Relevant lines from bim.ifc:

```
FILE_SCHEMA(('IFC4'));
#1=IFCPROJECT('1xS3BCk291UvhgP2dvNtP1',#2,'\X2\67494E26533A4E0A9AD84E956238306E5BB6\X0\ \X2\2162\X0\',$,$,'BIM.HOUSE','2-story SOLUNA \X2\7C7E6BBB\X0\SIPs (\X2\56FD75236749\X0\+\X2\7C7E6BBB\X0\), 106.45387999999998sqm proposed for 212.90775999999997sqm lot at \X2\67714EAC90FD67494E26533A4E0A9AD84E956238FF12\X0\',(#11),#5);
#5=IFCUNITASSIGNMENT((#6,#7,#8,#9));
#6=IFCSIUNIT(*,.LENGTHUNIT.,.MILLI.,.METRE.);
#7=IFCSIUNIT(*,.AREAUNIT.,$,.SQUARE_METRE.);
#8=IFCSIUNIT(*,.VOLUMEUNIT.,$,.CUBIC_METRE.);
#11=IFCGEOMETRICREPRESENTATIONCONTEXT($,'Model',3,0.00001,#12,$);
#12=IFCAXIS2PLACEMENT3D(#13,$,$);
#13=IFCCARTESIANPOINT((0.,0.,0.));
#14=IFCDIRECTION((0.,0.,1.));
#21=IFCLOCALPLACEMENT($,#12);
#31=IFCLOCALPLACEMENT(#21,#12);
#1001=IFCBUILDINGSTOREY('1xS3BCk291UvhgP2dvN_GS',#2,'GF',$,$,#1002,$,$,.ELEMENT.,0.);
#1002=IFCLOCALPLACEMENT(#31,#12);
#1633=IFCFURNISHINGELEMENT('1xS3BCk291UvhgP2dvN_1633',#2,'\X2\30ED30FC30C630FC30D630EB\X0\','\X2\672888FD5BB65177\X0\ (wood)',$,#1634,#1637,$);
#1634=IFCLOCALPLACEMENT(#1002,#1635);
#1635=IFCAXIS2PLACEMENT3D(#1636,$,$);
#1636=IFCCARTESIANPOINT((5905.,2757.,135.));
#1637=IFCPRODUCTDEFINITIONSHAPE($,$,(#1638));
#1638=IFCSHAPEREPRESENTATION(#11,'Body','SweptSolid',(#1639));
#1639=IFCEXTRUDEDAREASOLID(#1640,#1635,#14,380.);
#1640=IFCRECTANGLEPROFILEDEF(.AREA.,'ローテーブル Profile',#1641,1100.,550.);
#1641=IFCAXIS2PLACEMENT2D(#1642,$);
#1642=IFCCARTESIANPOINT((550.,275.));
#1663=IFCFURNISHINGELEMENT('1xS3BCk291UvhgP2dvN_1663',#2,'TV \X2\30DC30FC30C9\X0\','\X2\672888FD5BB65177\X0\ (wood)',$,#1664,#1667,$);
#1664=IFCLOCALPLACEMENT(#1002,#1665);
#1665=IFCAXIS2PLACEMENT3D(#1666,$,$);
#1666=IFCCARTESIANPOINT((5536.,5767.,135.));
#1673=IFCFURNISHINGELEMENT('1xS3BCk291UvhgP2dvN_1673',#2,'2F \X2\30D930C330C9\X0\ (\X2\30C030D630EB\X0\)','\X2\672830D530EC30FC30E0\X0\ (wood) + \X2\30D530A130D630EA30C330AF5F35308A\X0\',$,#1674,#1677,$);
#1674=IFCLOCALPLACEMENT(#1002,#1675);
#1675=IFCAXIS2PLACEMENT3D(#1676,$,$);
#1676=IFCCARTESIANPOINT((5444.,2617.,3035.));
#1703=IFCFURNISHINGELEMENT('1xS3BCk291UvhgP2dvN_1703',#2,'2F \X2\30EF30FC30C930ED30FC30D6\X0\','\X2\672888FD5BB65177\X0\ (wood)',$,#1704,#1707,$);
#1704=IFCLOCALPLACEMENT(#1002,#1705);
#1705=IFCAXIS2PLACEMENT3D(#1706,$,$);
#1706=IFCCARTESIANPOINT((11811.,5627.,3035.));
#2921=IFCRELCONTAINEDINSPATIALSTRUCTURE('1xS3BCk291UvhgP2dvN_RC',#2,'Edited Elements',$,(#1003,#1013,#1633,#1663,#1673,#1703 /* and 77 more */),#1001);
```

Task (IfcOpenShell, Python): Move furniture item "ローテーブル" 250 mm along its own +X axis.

```python
import ifcopenshell
import ifcopenshell.api.geometry
import ifcopenshell.util.placement

model = ifcopenshell.open("bim.ifc")

item = model.by_id(1633)
matrix = ifcopenshell.util.placement.get_local_placement(item.ObjectPlacement)
matrix[:3, 3] += matrix[:3, 0] * 250.0
ifcopenshell.api.geometry.edit_object_placement(model, product=item, matrix=matrix, is_si=False)

print(ifcopenshell.util.placement.get_local_placement(item.ObjectPlacement).round(3) + 0.0)

model.write("bim_edited.ifc")
```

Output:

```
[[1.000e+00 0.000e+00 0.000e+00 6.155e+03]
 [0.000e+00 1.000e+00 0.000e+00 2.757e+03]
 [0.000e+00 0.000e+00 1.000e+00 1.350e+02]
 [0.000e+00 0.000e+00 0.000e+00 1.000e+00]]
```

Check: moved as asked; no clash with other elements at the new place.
